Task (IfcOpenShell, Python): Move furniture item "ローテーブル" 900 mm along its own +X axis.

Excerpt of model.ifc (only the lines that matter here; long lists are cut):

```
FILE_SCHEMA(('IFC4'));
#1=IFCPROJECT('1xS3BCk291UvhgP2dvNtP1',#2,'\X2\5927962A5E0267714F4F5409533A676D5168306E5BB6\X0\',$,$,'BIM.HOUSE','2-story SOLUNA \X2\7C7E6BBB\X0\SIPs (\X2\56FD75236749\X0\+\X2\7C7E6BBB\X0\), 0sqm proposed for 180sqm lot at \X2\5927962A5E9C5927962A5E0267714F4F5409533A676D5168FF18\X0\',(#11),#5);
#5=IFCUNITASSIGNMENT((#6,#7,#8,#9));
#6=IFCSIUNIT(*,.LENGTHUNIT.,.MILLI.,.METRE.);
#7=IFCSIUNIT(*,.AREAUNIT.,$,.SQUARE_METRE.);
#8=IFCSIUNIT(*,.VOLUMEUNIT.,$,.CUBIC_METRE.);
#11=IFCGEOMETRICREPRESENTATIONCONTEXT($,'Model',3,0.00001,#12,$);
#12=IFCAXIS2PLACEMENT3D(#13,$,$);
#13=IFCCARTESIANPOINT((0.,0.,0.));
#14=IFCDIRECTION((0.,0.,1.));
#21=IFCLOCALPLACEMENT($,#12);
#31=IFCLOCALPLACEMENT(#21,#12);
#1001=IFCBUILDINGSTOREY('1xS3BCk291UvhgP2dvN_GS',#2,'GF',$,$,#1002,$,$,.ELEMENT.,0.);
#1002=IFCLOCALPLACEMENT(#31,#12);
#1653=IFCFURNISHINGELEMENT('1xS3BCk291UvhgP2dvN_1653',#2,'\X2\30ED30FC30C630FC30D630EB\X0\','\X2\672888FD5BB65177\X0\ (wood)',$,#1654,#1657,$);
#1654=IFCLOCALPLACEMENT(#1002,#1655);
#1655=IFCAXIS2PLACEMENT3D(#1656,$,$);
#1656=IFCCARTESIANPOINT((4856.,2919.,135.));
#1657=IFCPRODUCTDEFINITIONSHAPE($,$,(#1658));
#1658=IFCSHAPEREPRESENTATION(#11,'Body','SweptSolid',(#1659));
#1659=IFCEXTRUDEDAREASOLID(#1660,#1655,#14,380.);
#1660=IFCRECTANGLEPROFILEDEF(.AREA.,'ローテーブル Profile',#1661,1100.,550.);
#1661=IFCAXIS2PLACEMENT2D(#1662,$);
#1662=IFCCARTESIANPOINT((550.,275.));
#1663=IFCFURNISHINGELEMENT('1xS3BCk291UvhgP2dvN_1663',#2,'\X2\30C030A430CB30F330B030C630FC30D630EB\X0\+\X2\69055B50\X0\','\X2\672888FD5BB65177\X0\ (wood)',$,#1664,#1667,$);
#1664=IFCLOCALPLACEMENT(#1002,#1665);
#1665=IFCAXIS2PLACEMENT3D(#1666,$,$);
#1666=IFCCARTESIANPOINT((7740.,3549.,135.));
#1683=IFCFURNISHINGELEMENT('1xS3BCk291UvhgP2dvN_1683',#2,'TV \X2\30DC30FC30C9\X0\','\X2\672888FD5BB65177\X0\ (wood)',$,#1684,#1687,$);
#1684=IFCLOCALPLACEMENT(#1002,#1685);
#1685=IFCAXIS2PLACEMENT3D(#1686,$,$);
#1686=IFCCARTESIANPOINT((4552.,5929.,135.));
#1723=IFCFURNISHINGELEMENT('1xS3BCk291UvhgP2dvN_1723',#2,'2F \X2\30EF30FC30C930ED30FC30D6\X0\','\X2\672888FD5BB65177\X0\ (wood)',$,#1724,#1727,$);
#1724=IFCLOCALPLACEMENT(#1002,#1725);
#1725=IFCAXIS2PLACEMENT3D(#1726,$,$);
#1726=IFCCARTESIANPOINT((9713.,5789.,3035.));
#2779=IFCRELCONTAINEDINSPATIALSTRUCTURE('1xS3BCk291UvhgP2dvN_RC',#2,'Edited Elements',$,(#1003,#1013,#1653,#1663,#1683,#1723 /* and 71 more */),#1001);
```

```python
import ifcopenshell
import ifcopenshell.api.geometry
import ifcopenshell.util.placement
import ifcopenshell.util.unit

model = ifcopenshell.open("model.ifc")
unit_scale = ifcopenshell.util.unit.calculate_unit_scale(model)

item = model.by_id(1653)
matrix = ifcopenshell.util.placement.get_local_placement(item.ObjectPlacement)
matrix[:3, 3] += matrix[:3, 0] * 0.9 / unit_scale
ifcopenshell.api.geometry.edit_object_placement(model, product=item, matrix=matrix, is_si=False)

print(ifcopenshell.util.placement.get_local_placement(item.ObjectPlacement).round(3) + 0.0)

model.write("model_v2.ifc")
```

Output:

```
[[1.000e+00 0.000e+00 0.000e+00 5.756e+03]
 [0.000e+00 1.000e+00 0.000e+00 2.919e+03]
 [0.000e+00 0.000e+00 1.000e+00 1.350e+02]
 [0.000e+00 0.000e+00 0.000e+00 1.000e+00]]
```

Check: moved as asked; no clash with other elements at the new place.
